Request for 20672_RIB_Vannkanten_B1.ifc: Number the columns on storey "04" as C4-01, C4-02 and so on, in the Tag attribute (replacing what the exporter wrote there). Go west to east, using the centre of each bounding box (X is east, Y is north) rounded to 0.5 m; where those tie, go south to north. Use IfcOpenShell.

First a look at what the model holds.

```python
import ifcopenshell
import ifcopenshell.util.element
import ifcopenshell.util.placement

model = ifcopenshell.open("20672_RIB_Vannkanten_B1.ifc")
print(model.schema)
storey = next(s for s in model.by_type("IfcBuildingStorey") if s.Name == "04")
columns = [e for e in ifcopenshell.util.element.get_decomposition(storey) if e.is_a("IfcColumn")]
for e in sorted(columns, key=lambda e: e.id()):
    origin = ifcopenshell.util.placement.get_local_placement(e.ObjectPlacement)[:3, 3]
    print(e.id(), e.Tag, e.Name, origin.round(2) + 0.0, sep=" | ")
```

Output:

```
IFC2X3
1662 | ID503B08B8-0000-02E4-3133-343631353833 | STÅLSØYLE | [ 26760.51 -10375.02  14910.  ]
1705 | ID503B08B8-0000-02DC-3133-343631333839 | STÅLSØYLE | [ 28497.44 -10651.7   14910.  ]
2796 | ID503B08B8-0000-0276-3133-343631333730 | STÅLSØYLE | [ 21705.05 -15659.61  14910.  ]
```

```python
import ifcopenshell
import ifcopenshell.geom
import ifcopenshell.util.element
import ifcopenshell.util.shape

model = ifcopenshell.open("20672_RIB_Vannkanten_B1.ifc")
settings = ifcopenshell.geom.settings()
settings.set("use-world-coords", True)


def centre(element):
    shape = ifcopenshell.geom.create_shape(settings, element)
    return ifcopenshell.util.shape.get_bbox_centroid(shape.geometry)


storey = next(s for s in model.by_type("IfcBuildingStorey") if s.Name == "04")
columns = [e for e in ifcopenshell.util.element.get_decomposition(storey) if e.is_a("IfcColumn")]

# Insertion points can sit at a corner or the storey origin, so sort by the geometry (in metres).
centres = {e: centre(e) for e in columns}
columns.sort(key=lambda e: (round(centres[e][0] / 0.5), centres[e][1]))

for i, e in enumerate(columns, start=1):
    number = f"C4-{i:02d}"
    e.Tag = number
    print(e.id(), number)

model.write("20672_RIB_Vannkanten_B1_updated.ifc")
```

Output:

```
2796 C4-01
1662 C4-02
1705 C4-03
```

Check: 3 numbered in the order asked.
